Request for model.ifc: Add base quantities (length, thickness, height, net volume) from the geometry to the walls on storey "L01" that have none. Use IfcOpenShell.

First a look at what the model holds.

```python
import ifcopenshell
import ifcopenshell.util.element
import ifcopenshell.util.unit

model = ifcopenshell.open("model.ifc")
print(model.schema)
for unit_type in ("LENGTHUNIT", "AREAUNIT", "VOLUMEUNIT"):
    print(unit_type, ifcopenshell.util.unit.calculate_unit_scale(model, unit_type))
storey = next(s for s in model.by_type("IfcBuildingStorey") if s.Name == "L01")
walls = [e for e in ifcopenshell.util.element.get_decomposition(storey) if e.is_a("IfcWall")]
for e in sorted(walls, key=lambda e: e.id()):
    print(e.id(), e.is_a(), e.Name, list(ifcopenshell.util.element.get_psets(e, qtos_only=True)), sep=" | ")
```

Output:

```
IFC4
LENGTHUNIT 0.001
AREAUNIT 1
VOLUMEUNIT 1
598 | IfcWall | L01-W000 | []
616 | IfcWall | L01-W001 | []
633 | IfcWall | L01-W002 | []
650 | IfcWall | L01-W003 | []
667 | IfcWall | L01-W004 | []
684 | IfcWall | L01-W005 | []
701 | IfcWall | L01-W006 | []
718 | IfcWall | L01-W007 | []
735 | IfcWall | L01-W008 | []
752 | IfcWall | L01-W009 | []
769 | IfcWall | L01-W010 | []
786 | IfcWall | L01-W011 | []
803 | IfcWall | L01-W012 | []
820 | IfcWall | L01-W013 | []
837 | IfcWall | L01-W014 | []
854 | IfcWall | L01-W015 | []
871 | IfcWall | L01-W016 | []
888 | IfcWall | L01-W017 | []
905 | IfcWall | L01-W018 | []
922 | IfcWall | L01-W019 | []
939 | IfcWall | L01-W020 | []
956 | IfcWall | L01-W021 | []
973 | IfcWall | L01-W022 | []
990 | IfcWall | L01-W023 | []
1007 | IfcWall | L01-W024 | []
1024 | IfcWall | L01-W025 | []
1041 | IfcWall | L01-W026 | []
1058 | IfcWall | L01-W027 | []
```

```python
import ifcopenshell
import ifcopenshell.api.pset
import ifcopenshell.geom
import ifcopenshell.util.element
import ifcopenshell.util.shape
import ifcopenshell.util.unit

model = ifcopenshell.open("model.ifc")
unit_scale = ifcopenshell.util.unit.calculate_unit_scale(model)
volume_scale = ifcopenshell.util.unit.calculate_unit_scale(model, "VOLUMEUNIT")
settings = ifcopenshell.geom.settings()

storey = next(s for s in model.by_type("IfcBuildingStorey") if s.Name == "L01")
walls = [e for e in ifcopenshell.util.element.get_decomposition(storey) if e.is_a("IfcWall")]

for e in sorted(walls, key=lambda e: e.id()):
    if ifcopenshell.util.element.get_psets(e, qtos_only=True, should_inherit=False):
        continue
    # Geometry comes back in metres, in the element's own axes.
    shape = ifcopenshell.geom.create_shape(settings, e)
    values = {
        "Length": ifcopenshell.util.shape.get_x(shape.geometry) / unit_scale,
        "Width": ifcopenshell.util.shape.get_y(shape.geometry) / unit_scale,
        "Height": ifcopenshell.util.shape.get_z(shape.geometry) / unit_scale,
        "NetVolume": ifcopenshell.util.shape.get_volume(shape.geometry) / volume_scale,
    }
    qto = ifcopenshell.api.pset.add_qto(model, product=e, name="Qto_WallBaseQuantities")
    ifcopenshell.api.pset.edit_qto(model, qto=qto, properties=values)
    print(e.id(), {k: round(v, 3) for k, v in values.items()})

model.write("model_v2.ifc")
```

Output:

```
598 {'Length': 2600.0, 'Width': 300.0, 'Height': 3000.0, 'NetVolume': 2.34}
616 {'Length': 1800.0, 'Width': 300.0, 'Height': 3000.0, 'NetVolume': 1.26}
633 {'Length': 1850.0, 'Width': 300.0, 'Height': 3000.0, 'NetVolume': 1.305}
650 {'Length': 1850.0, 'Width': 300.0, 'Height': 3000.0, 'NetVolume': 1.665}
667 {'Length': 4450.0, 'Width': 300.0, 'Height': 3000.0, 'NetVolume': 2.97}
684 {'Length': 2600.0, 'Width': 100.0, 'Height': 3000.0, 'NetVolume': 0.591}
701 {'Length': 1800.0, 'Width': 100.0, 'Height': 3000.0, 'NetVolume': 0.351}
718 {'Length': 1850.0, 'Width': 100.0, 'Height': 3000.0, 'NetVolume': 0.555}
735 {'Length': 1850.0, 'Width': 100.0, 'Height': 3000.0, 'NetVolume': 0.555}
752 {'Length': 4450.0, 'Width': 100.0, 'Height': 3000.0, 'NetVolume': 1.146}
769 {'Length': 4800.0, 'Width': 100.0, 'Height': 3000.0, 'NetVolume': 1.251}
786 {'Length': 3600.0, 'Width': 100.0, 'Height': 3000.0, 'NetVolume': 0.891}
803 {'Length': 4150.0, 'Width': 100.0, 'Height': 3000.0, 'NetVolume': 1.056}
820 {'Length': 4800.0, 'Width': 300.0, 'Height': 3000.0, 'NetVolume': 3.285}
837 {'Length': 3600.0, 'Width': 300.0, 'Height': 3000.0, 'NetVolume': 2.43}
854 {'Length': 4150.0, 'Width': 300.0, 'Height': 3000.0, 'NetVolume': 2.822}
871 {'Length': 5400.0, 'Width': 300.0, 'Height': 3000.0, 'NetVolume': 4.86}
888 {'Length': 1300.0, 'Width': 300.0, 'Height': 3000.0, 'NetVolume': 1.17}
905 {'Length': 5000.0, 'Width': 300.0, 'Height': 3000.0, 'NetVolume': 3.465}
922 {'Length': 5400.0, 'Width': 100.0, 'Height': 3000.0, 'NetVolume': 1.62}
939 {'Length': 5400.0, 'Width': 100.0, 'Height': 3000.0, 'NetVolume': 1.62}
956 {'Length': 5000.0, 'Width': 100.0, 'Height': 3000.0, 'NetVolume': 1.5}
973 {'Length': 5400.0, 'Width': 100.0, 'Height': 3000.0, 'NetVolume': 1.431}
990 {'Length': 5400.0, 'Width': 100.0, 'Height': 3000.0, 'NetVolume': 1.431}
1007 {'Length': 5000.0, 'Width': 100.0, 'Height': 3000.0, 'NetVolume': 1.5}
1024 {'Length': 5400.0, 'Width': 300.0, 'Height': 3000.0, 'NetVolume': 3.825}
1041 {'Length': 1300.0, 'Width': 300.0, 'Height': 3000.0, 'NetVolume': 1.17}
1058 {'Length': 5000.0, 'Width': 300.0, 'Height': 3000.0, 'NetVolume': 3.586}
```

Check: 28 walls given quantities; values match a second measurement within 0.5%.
